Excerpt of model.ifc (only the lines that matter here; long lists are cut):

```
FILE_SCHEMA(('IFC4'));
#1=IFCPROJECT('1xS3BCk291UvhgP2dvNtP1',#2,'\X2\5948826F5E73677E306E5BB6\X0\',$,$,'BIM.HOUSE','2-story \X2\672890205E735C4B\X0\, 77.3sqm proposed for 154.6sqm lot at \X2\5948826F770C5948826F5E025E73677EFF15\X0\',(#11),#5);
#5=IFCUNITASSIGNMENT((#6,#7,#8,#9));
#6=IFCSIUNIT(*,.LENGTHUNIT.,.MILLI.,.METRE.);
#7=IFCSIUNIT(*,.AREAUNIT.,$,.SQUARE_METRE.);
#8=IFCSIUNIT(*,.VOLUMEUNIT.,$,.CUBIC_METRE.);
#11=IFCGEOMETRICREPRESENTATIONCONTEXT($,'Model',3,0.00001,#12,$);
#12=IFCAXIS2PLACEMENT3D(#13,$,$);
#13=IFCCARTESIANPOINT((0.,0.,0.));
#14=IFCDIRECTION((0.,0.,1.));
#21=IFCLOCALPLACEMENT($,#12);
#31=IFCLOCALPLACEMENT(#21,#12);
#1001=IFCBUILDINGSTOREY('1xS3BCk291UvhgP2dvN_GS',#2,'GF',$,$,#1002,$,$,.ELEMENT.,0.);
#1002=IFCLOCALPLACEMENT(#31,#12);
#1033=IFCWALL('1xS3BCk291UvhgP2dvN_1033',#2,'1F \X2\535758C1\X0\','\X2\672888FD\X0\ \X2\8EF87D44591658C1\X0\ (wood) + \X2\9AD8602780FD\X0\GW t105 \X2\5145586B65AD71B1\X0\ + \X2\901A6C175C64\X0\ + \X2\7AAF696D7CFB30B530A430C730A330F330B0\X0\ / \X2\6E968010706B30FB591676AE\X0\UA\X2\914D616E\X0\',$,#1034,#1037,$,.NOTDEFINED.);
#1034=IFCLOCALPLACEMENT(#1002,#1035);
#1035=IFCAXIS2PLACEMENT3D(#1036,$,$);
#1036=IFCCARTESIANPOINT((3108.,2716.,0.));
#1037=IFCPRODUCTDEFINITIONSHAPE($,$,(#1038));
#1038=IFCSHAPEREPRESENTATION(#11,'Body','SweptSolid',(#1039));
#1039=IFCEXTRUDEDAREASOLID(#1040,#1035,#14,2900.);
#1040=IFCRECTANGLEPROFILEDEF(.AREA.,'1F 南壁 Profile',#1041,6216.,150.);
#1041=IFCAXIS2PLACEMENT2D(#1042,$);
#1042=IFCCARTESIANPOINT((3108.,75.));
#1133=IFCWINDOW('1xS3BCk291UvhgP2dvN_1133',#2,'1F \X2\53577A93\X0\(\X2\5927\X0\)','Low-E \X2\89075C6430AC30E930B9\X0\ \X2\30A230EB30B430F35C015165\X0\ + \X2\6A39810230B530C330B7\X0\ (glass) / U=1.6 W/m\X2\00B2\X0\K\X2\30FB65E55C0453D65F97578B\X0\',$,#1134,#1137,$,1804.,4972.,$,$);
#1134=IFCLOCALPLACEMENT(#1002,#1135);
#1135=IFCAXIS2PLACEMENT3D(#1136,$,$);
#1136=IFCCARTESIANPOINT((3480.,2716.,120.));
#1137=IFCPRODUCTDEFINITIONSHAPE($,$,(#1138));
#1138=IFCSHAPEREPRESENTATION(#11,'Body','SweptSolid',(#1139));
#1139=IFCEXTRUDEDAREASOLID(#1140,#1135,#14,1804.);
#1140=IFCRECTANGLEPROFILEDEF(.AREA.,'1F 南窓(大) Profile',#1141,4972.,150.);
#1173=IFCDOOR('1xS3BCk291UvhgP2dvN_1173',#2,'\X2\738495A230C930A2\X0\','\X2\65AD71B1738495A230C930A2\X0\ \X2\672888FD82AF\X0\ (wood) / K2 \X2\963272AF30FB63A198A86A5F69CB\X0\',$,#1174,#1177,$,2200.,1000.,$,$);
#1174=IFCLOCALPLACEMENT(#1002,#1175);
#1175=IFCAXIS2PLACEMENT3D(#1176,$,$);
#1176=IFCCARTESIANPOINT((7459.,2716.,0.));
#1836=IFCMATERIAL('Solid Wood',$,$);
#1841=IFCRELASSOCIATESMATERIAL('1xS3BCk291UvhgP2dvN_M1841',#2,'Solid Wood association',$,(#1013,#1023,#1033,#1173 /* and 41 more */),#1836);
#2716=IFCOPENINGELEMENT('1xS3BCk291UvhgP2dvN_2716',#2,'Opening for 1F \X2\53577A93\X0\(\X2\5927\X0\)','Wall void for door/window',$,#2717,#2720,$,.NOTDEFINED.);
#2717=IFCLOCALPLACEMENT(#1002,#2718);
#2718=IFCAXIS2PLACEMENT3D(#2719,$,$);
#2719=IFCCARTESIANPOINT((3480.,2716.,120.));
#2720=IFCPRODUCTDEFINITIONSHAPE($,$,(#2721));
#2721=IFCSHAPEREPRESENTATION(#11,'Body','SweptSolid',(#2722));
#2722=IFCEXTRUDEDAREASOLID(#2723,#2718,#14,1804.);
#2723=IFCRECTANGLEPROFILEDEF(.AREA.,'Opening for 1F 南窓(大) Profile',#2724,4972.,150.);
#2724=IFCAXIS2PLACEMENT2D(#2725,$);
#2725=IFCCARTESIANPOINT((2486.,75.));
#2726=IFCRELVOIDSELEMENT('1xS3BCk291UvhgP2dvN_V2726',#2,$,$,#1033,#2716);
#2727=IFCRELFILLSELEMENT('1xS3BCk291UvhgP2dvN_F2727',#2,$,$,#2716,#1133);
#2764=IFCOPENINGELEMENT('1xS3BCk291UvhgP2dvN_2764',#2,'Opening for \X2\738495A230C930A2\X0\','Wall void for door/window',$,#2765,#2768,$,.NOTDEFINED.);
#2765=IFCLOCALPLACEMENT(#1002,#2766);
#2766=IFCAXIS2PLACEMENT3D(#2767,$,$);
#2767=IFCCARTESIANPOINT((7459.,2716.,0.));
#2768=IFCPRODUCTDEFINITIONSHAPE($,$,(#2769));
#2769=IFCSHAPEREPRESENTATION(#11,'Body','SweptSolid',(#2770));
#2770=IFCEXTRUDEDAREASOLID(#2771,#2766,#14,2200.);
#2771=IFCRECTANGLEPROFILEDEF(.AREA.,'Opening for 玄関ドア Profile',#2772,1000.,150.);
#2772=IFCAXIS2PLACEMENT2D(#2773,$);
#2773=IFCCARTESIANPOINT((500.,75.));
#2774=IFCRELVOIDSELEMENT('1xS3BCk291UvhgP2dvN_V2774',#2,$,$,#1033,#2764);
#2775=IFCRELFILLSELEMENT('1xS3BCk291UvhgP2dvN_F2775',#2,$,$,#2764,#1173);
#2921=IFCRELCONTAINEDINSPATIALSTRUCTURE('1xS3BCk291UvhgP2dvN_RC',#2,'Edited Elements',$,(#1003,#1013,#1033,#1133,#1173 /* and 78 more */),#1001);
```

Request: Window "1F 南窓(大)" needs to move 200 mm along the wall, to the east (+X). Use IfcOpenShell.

```python
import ifcopenshell
import ifcopenshell.api.geometry
import ifcopenshell.util.placement

model = ifcopenshell.open("model.ifc")

window = model.by_id(1133)
opening = window.FillsVoids[0].RelatingOpeningElement
wall = opening.VoidsElements[0].RelatingBuildingElement

wall_matrix = ifcopenshell.util.placement.get_local_placement(wall.ObjectPlacement)
shift = wall_matrix[:3, 0] * 200.0
before = ifcopenshell.util.placement.get_local_placement(window.ObjectPlacement)[:3, 3].copy()

# The window is not placed relative to its opening, so move both.
for product in (opening, window):
    matrix = ifcopenshell.util.placement.get_local_placement(product.ObjectPlacement)
    matrix[:3, 3] += shift
    ifcopenshell.api.geometry.edit_object_placement(model, product=product, matrix=matrix, is_si=False)

after = ifcopenshell.util.placement.get_local_placement(window.ObjectPlacement)[:3, 3]
print("window moved by", (after - before).round(3) + 0.0)

model.write("model_updated.ifc")
```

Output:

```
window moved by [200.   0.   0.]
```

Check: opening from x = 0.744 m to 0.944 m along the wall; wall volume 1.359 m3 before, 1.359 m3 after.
